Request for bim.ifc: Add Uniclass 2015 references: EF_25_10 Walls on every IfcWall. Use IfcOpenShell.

First a look at what the model holds.

```python
import ifcopenshell

model = ifcopenshell.open("bim.ifc")
print(model.schema)
print("classifications:", [c.Name for c in model.by_type("IfcClassification")])
for ifc_class in ("IfcDoor", "IfcRoof", "IfcStair", "IfcWall", "IfcWindow"):
    print(ifc_class, len(model.by_type(ifc_class)))
```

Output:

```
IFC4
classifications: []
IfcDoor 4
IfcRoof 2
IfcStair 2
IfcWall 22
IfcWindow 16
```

```python
import ifcopenshell
import ifcopenshell.api.classification

model = ifcopenshell.open("bim.ifc")

system = ifcopenshell.api.classification.add_classification(model, classification="Uniclass 2015")

codes = {
    "IfcWall": ("EF_25_10", "Walls"),
}
for ifc_class, (code, name) in codes.items():
    products = model.by_type(ifc_class)
    ifcopenshell.api.classification.add_reference(
        model, products=products, classification=system, identification=code, name=name
    )
    print(code, len(products))

model.write("bim_v2.ifc")
```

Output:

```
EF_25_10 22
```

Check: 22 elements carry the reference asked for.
